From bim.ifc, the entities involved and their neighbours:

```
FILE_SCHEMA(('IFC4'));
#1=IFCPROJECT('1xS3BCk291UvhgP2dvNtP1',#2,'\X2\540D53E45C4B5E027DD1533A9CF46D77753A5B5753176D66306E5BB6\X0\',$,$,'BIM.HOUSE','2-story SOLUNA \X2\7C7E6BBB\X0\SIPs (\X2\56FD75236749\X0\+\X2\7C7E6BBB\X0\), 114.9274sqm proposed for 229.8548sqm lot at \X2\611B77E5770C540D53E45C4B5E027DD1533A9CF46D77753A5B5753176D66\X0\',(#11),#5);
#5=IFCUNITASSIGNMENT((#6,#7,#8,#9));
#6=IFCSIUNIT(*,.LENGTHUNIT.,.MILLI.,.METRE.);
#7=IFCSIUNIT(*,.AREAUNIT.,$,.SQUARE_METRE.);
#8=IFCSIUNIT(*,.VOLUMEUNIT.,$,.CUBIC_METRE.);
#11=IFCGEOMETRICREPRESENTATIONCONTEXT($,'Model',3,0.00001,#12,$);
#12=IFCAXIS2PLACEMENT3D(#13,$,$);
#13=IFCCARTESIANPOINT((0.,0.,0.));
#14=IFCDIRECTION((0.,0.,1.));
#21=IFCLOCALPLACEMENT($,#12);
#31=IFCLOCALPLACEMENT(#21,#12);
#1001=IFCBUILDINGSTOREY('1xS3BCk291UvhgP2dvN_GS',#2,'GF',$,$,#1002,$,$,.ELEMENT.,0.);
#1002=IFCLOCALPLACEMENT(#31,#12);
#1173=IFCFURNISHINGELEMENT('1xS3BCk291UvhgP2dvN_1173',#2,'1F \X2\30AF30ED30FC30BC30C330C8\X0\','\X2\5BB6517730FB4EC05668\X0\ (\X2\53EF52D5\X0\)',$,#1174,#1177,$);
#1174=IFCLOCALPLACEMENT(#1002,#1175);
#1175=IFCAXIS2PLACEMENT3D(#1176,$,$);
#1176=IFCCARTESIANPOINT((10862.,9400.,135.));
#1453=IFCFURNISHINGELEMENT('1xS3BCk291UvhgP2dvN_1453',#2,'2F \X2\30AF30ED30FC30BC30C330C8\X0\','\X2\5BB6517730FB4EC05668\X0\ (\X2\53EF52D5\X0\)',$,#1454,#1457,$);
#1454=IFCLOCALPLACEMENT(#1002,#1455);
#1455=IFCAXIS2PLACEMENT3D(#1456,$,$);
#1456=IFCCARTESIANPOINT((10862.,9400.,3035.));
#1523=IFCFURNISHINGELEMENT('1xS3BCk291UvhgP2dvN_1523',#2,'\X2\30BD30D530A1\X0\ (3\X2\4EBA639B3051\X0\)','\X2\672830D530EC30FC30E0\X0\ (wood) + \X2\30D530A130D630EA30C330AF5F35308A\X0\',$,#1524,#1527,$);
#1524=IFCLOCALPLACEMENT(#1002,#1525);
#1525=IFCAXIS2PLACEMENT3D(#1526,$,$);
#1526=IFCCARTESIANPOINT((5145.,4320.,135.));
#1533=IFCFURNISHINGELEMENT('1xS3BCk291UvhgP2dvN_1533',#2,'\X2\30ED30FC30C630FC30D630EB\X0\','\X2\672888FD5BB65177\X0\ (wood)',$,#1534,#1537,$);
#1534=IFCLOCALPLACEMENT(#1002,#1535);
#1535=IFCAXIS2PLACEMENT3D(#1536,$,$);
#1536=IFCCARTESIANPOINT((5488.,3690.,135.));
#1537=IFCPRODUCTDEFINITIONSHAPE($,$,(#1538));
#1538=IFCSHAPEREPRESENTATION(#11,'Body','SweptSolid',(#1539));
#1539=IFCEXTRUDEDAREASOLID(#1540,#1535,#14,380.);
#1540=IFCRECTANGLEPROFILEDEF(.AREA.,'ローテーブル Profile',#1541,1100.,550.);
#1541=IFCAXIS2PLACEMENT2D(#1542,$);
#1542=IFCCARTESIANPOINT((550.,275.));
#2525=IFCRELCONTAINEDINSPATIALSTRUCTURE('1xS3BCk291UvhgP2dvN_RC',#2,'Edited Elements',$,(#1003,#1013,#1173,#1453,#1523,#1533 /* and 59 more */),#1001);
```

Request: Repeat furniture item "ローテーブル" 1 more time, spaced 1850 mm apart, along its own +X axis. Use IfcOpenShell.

```python
import ifcopenshell
import ifcopenshell.api.geometry
import ifcopenshell.api.root
import ifcopenshell.util.element
import ifcopenshell.util.placement

model = ifcopenshell.open("bim.ifc")


def reuse_history(source, copy):
    """copy_class also copies each property set's owner history, people and application; keep the originals."""
    for rel in copy.IsDefinedBy:
        if rel.is_a("IfcRelDefinesByProperties") and (history := rel.RelatingPropertyDefinition.OwnerHistory):
            rel.RelatingPropertyDefinition.OwnerHistory = source.OwnerHistory
            ifcopenshell.util.element.remove_deep2(model, history)


source = model.by_guid("1xS3BCk291UvhgP2dvN_1533")
base = ifcopenshell.util.placement.get_local_placement(source.ObjectPlacement)
step = base[:3, 0] * 1850.0

for i in range(1, 2):
    copy = ifcopenshell.api.root.copy_class(model, product=source)
    copy.Representation = ifcopenshell.util.element.copy_deep(
        model, source.Representation, exclude=["IfcGeometricRepresentationContext", "IfcRepresentationMap"]
    )
    reuse_history(source, copy)
    matrix = base.copy()
    matrix[:3, 3] += i * step
    print("added at", matrix[:3, 3].round(3) + 0.0)
    ifcopenshell.api.geometry.edit_object_placement(model, product=copy, matrix=matrix, is_si=False)

model.write("bim_v2.ifc")
```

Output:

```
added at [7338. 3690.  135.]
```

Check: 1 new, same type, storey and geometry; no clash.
